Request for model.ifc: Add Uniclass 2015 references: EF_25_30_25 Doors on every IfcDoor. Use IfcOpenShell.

First a look at what the model holds.

```python
import ifcopenshell

model = ifcopenshell.open("model.ifc")
print(model.schema)
print("classifications:", [c.Name for c in model.by_type("IfcClassification")])
for ifc_class in ("IfcDoor", "IfcRoof", "IfcStair", "IfcWall", "IfcWindow"):
    print(ifc_class, len(model.by_type(ifc_class)))
```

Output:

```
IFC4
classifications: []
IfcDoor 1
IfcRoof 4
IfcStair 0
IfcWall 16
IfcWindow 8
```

```python
import ifcopenshell
import ifcopenshell.api.classification

model = ifcopenshell.open("model.ifc")

system = ifcopenshell.api.classification.add_classification(model, classification="Uniclass 2015")

codes = {
    "IfcDoor": ("EF_25_30_25", "Doors"),
}
for ifc_class, (code, name) in codes.items():
    products = model.by_type(ifc_class)
    ifcopenshell.api.classification.add_reference(
        model, products=products, classification=system, identification=code, name=name
    )
    print(code, len(products))

model.write("model_edited.ifc")
```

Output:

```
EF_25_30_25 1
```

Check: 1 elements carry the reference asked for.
